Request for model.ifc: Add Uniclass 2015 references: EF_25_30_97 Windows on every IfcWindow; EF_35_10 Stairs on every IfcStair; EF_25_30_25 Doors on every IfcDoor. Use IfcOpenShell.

First a look at what the model holds.

```python
import ifcopenshell

model = ifcopenshell.open("model.ifc")
print(model.schema)
print("classifications:", [c.Name for c in model.by_type("IfcClassification")])
for ifc_class in ("IfcDoor", "IfcRoof", "IfcStair", "IfcWall", "IfcWindow"):
    print(ifc_class, len(model.by_type(ifc_class)))
```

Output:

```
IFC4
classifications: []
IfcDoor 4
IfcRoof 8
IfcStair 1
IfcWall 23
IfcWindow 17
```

```python
import ifcopenshell
import ifcopenshell.api.classification

model = ifcopenshell.open("model.ifc")

system = ifcopenshell.api.classification.add_classification(model, classification="Uniclass 2015")

codes = {
    "IfcWindow": ("EF_25_30_97", "Windows"),
    "IfcStair": ("EF_35_10", "Stairs"),
    "IfcDoor": ("EF_25_30_25", "Doors"),
}
for ifc_class, (code, name) in codes.items():
    products = model.by_type(ifc_class)
    ifcopenshell.api.classification.add_reference(
        model, products=products, classification=system, identification=code, name=name
    )
    print(code, len(products))

model.write("model_v2.ifc")
```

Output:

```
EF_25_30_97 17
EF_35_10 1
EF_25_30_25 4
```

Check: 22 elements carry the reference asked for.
